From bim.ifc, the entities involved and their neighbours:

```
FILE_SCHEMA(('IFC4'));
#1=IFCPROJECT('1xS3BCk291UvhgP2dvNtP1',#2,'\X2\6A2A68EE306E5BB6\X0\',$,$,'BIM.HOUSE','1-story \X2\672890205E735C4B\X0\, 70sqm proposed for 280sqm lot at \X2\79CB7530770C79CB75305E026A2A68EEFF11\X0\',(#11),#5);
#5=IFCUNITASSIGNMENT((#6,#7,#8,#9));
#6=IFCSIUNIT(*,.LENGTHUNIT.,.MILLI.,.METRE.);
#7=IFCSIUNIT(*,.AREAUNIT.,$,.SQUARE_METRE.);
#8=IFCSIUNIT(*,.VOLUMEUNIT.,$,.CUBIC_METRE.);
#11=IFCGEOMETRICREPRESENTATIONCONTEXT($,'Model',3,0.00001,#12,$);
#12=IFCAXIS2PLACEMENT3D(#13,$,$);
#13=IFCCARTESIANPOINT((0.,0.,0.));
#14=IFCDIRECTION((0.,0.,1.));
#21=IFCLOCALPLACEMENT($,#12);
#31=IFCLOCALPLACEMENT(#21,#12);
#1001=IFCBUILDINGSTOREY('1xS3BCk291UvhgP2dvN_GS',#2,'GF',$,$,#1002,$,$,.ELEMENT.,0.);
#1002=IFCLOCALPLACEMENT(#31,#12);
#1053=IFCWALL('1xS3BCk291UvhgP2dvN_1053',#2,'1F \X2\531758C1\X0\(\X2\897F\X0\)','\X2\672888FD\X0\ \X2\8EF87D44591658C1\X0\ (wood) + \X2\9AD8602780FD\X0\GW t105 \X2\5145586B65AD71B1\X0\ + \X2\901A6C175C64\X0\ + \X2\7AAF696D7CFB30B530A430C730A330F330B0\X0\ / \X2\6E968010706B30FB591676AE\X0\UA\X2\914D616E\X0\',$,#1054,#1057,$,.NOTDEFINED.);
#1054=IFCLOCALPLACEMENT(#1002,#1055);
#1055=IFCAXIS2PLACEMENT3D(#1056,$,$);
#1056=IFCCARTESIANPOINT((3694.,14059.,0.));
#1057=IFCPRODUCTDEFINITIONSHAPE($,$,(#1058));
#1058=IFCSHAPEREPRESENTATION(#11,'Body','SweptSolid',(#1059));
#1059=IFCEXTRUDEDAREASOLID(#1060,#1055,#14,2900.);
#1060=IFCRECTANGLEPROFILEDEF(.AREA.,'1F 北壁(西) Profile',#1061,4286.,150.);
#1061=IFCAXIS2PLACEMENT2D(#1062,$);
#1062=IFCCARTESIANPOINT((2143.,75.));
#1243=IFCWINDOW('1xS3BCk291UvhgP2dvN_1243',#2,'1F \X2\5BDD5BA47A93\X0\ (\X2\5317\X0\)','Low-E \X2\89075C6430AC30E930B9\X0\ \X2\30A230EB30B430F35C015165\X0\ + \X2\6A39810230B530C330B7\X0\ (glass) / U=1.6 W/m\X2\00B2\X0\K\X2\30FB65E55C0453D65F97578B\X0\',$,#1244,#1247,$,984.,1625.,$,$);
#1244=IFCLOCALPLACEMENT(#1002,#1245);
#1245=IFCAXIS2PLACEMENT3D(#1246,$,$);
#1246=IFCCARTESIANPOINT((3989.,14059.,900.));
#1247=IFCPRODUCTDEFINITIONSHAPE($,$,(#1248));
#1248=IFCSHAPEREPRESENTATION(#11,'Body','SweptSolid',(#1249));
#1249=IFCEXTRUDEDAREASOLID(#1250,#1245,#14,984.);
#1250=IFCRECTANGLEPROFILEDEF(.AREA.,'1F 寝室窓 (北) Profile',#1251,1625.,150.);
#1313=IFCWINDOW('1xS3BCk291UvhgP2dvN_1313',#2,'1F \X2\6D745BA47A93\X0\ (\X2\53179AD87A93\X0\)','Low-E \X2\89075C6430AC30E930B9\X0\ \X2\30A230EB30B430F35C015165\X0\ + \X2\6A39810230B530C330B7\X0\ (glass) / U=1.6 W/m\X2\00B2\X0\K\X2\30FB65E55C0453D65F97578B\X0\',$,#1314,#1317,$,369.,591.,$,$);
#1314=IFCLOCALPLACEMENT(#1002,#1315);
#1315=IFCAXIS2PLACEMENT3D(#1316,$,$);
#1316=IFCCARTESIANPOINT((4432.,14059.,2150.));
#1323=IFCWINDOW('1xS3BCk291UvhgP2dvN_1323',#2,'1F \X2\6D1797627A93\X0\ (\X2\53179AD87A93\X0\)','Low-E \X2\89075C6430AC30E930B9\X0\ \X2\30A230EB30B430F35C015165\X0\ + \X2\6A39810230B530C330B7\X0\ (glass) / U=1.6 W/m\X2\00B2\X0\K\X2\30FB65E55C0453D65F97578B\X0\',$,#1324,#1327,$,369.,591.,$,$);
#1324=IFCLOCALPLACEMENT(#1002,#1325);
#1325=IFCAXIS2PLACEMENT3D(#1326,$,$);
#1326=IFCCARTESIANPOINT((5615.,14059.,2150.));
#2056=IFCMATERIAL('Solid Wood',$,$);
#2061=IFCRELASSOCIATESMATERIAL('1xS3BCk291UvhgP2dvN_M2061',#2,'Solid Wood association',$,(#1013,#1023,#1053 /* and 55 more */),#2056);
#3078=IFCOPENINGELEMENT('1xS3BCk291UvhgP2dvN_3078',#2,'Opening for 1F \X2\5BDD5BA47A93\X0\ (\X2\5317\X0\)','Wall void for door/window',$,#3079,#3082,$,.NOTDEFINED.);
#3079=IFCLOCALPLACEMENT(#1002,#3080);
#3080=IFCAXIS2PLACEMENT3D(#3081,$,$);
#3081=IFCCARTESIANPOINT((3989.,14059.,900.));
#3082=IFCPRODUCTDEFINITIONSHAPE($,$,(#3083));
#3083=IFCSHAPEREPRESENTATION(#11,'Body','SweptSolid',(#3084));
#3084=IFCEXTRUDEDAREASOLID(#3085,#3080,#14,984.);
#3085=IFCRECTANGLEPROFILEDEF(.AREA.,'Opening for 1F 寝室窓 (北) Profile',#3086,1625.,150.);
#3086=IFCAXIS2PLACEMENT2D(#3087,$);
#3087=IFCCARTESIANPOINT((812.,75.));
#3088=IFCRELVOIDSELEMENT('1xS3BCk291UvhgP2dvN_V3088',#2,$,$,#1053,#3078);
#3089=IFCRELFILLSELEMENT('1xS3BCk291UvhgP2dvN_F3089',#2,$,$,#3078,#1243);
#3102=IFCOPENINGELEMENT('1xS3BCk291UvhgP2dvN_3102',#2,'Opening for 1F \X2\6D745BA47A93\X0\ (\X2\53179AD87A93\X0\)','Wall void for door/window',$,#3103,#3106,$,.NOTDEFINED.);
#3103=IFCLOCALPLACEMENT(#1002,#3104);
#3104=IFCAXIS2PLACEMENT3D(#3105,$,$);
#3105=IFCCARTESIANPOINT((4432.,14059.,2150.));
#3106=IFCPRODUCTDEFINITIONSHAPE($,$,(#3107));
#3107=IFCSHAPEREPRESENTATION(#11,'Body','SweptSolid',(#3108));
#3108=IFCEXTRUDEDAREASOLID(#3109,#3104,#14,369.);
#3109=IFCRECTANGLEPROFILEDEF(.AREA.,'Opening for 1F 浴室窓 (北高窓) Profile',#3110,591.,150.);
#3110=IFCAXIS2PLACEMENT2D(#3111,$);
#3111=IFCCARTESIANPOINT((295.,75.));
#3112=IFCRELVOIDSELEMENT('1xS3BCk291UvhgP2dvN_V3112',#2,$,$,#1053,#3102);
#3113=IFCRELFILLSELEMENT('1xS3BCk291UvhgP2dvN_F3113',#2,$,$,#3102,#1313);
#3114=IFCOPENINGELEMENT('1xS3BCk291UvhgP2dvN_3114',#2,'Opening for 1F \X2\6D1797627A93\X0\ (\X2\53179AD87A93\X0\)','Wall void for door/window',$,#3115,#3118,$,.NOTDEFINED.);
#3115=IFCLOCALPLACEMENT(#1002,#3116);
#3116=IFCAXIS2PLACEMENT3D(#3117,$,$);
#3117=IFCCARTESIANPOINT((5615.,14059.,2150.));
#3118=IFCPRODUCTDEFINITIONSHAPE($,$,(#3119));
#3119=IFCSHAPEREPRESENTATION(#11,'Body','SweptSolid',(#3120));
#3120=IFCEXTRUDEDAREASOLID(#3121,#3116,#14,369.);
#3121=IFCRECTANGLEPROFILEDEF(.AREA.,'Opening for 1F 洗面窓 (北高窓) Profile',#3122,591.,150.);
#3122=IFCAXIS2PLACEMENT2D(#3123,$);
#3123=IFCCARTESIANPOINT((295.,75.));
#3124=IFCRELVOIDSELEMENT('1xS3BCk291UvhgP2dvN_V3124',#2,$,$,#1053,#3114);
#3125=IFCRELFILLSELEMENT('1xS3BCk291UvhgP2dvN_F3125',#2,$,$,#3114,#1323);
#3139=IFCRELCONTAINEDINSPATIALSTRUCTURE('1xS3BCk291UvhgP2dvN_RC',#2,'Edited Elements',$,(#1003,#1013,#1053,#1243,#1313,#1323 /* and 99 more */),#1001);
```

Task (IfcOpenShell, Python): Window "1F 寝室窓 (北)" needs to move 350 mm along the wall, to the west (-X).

```python
import ifcopenshell
import ifcopenshell.api.geometry
import ifcopenshell.util.placement
import ifcopenshell.util.unit

model = ifcopenshell.open("bim.ifc")
unit_scale = ifcopenshell.util.unit.calculate_unit_scale(model)

window = model.by_guid("1xS3BCk291UvhgP2dvN_1243")
opening = window.FillsVoids[0].RelatingOpeningElement
wall = opening.VoidsElements[0].RelatingBuildingElement

wall_matrix = ifcopenshell.util.placement.get_local_placement(wall.ObjectPlacement)
shift = wall_matrix[:3, 0] * -0.35 / unit_scale
before = ifcopenshell.util.placement.get_local_placement(window.ObjectPlacement)[:3, 3].copy()

# The window is not placed relative to its opening, so move both.
for product in (opening, window):
    matrix = ifcopenshell.util.placement.get_local_placement(product.ObjectPlacement)
    matrix[:3, 3] += shift
    ifcopenshell.api.geometry.edit_object_placement(model, product=product, matrix=matrix, is_si=False)

after = ifcopenshell.util.placement.get_local_placement(window.ObjectPlacement)[:3, 3]
print("window moved by", (after - before).round(3) + 0.0)

model.write("bim_updated.ifc")
```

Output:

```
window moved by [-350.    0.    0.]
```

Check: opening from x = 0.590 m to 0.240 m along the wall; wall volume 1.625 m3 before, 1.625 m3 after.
